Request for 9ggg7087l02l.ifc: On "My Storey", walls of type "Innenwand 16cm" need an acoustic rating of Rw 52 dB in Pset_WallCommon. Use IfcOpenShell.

First a look at what the model holds.

```python
import ifcopenshell
import ifcopenshell.util.element

model = ifcopenshell.open("9ggg7087l02l.ifc")
print(model.schema)
storey = next(s for s in model.by_type("IfcBuildingStorey") if s.Name == "My Storey")
walls = [e for e in ifcopenshell.util.element.get_decomposition(storey) if e.is_a("IfcWall")]
seen = {}
for e in walls:
    element_type = ifcopenshell.util.element.get_type(e)
    key = (element_type.Name if element_type != e and element_type else None, ifcopenshell.util.element.get_pset(e, "Pset_WallCommon", "AcousticRating"))
    seen[key] = seen.get(key, 0) + 1
for (name, value), count in sorted(seen.items(), key=str):
    print(count, "x", name, "|", value)
```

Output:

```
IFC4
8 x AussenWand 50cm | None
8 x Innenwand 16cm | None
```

```python
import ifcopenshell
import ifcopenshell.api.pset
import ifcopenshell.util.element

model = ifcopenshell.open("9ggg7087l02l.ifc")

storey = next(s for s in model.by_type("IfcBuildingStorey") if s.Name == "My Storey")
walls = [e for e in ifcopenshell.util.element.get_decomposition(storey) if e.is_a("IfcWall")]

count = 0
for e in walls:
    element_type = ifcopenshell.util.element.get_type(e)
    if element_type in (None, e) or element_type.Name != "Innenwand 16cm":
        continue
    # add_pset returns the element's existing set when there is one.
    pset = ifcopenshell.api.pset.add_pset(model, product=e, name="Pset_WallCommon")
    ifcopenshell.api.pset.edit_pset(model, pset=pset, properties={"AcousticRating": "Rw 52 dB"})
    count += 1

print(count, "walls updated")

model.write("9ggg7087l02l-out.ifc")
```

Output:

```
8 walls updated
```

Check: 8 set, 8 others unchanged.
